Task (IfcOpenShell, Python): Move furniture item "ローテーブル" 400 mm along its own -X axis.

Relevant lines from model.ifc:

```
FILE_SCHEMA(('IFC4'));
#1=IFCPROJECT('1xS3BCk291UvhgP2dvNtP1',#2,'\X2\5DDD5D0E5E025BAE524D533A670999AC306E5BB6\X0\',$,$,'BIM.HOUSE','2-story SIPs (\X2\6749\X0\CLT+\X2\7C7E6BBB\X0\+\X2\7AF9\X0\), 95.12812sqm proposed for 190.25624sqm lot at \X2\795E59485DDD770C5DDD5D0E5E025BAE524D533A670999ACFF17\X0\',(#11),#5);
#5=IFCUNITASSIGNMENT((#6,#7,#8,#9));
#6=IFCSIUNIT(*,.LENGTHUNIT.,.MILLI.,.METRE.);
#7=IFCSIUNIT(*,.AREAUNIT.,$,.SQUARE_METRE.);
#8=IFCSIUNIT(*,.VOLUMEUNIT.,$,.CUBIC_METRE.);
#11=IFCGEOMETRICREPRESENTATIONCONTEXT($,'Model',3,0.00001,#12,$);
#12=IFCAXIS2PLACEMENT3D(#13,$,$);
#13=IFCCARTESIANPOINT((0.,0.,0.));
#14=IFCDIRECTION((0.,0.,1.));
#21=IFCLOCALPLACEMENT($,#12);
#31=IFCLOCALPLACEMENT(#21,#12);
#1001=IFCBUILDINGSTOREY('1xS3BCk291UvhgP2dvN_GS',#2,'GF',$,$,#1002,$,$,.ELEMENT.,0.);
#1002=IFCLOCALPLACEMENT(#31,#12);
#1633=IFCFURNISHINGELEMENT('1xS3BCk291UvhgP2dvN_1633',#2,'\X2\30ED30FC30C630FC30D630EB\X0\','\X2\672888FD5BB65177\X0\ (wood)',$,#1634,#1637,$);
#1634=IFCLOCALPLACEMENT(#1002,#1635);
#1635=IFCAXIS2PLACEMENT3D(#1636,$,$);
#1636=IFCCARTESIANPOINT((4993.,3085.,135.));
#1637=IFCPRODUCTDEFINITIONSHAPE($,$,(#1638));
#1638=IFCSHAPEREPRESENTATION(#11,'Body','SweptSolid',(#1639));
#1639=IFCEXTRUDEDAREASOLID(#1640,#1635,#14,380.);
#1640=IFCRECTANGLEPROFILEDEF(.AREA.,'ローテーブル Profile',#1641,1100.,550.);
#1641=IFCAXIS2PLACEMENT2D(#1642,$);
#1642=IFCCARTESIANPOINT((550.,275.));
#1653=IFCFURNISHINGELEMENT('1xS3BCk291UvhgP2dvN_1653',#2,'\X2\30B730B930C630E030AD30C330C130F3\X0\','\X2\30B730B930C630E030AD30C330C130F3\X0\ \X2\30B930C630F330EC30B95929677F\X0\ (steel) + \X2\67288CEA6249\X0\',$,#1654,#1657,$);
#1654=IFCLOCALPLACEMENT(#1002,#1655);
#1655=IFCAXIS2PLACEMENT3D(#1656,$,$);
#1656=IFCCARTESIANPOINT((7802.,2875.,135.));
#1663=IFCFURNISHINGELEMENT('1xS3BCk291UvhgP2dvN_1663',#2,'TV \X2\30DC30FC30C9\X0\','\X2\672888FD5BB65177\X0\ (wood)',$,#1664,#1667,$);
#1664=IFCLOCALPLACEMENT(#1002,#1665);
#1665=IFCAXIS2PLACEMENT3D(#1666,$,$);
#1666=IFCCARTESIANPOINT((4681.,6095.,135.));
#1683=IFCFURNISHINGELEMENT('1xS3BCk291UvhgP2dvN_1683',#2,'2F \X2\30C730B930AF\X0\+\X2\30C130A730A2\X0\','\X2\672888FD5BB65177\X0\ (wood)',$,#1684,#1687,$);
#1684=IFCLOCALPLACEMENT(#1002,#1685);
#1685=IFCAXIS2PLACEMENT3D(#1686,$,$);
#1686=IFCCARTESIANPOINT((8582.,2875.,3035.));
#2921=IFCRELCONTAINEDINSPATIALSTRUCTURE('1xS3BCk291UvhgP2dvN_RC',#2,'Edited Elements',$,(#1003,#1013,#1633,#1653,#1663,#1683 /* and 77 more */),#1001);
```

```python
import ifcopenshell
import ifcopenshell.api.geometry
import ifcopenshell.util.placement
import ifcopenshell.util.unit

model = ifcopenshell.open("model.ifc")
unit_scale = ifcopenshell.util.unit.calculate_unit_scale(model)

item = model.by_guid("1xS3BCk291UvhgP2dvN_1633")
matrix = ifcopenshell.util.placement.get_local_placement(item.ObjectPlacement)
matrix[:3, 3] -= matrix[:3, 0] * 0.4 / unit_scale
ifcopenshell.api.geometry.edit_object_placement(model, product=item, matrix=matrix, is_si=False)

print(ifcopenshell.util.placement.get_local_placement(item.ObjectPlacement).round(3) + 0.0)

model.write("model-out.ifc")
```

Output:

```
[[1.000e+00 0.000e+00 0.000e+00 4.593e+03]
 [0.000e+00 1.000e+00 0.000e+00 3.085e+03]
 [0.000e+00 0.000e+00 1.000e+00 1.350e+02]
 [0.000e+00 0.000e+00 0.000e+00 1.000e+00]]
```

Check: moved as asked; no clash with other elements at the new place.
